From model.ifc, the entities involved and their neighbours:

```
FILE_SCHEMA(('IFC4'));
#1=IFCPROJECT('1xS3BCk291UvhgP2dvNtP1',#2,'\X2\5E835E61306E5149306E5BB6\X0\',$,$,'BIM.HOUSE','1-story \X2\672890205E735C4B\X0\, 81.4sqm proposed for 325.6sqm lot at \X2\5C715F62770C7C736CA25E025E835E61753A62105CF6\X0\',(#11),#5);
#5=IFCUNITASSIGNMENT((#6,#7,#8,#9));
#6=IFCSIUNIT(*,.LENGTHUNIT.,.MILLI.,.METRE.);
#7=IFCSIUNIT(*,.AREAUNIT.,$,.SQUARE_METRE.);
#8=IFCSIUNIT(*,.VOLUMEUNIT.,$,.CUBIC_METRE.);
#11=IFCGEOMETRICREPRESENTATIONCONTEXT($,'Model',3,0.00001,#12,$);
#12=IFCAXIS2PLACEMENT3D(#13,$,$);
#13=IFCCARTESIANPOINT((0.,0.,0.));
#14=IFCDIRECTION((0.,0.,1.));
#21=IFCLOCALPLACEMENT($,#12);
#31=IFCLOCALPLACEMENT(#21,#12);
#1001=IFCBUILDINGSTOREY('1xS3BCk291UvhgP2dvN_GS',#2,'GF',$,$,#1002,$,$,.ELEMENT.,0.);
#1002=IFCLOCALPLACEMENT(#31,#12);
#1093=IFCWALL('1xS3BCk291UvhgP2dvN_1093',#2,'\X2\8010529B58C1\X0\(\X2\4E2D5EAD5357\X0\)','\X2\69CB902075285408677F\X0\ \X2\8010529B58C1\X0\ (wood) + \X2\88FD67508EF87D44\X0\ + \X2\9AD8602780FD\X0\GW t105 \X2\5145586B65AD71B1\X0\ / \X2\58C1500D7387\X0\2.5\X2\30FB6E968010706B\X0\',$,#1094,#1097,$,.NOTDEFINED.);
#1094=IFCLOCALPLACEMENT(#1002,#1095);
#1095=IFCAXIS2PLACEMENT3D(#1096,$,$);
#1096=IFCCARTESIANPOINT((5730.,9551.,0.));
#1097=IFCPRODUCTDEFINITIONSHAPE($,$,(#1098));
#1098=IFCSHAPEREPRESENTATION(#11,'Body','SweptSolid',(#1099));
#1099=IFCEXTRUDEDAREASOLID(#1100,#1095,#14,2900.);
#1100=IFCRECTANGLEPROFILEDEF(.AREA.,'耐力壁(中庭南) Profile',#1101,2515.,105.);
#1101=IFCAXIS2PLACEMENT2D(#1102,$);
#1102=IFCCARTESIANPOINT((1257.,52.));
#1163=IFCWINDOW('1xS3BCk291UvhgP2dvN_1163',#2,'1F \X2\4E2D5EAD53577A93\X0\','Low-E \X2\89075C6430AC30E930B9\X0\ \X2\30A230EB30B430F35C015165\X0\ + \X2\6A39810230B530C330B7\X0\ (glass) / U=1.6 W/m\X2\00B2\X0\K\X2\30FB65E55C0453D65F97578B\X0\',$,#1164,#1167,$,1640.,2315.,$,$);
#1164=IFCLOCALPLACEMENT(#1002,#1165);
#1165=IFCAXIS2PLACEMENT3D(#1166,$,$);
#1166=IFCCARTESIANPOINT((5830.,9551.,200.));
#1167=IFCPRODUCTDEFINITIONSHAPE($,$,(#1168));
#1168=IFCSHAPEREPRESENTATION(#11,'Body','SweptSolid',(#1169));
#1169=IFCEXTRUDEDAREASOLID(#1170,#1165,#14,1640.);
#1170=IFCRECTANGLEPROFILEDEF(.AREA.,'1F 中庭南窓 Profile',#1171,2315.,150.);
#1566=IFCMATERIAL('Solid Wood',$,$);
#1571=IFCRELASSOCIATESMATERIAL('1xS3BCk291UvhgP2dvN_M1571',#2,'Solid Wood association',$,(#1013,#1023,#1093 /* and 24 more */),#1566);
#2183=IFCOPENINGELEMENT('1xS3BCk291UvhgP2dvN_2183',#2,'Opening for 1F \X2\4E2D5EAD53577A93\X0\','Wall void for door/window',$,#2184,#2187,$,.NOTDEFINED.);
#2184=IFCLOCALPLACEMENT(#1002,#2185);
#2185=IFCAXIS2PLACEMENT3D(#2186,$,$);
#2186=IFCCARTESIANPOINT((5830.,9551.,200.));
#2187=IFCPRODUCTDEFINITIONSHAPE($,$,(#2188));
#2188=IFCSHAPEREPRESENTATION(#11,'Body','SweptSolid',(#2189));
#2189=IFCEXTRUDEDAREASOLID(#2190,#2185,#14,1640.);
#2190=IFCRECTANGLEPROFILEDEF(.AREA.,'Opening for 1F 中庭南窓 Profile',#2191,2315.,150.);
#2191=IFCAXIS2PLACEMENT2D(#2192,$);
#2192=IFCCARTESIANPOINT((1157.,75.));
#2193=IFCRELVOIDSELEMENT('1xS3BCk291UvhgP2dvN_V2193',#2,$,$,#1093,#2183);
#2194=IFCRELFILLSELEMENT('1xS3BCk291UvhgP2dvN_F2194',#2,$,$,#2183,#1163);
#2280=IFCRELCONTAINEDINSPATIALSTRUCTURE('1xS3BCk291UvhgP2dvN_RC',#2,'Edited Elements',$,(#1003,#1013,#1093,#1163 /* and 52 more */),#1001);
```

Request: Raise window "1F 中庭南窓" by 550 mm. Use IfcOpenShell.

```python
import numpy as np
import ifcopenshell
import ifcopenshell.api.geometry
import ifcopenshell.util.placement
import ifcopenshell.util.unit

model = ifcopenshell.open("model.ifc")
unit_scale = ifcopenshell.util.unit.calculate_unit_scale(model)

window = model.by_guid("1xS3BCk291UvhgP2dvN_1163")
opening = window.FillsVoids[0].RelatingOpeningElement
dz = 0.55 / unit_scale

shift = np.array([0.0, 0.0, dz])
# The window is not placed relative to its opening, so move both.
for product in (opening, window):
    matrix = ifcopenshell.util.placement.get_local_placement(product.ObjectPlacement)
    matrix[:3, 3] += shift
    ifcopenshell.api.geometry.edit_object_placement(model, product=product, matrix=matrix, is_si=False)

print(f"moved by {dz * unit_scale:+.3f} m")

model.write("model_edited.ifc")
```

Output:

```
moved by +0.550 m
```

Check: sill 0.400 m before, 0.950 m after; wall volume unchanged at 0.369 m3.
